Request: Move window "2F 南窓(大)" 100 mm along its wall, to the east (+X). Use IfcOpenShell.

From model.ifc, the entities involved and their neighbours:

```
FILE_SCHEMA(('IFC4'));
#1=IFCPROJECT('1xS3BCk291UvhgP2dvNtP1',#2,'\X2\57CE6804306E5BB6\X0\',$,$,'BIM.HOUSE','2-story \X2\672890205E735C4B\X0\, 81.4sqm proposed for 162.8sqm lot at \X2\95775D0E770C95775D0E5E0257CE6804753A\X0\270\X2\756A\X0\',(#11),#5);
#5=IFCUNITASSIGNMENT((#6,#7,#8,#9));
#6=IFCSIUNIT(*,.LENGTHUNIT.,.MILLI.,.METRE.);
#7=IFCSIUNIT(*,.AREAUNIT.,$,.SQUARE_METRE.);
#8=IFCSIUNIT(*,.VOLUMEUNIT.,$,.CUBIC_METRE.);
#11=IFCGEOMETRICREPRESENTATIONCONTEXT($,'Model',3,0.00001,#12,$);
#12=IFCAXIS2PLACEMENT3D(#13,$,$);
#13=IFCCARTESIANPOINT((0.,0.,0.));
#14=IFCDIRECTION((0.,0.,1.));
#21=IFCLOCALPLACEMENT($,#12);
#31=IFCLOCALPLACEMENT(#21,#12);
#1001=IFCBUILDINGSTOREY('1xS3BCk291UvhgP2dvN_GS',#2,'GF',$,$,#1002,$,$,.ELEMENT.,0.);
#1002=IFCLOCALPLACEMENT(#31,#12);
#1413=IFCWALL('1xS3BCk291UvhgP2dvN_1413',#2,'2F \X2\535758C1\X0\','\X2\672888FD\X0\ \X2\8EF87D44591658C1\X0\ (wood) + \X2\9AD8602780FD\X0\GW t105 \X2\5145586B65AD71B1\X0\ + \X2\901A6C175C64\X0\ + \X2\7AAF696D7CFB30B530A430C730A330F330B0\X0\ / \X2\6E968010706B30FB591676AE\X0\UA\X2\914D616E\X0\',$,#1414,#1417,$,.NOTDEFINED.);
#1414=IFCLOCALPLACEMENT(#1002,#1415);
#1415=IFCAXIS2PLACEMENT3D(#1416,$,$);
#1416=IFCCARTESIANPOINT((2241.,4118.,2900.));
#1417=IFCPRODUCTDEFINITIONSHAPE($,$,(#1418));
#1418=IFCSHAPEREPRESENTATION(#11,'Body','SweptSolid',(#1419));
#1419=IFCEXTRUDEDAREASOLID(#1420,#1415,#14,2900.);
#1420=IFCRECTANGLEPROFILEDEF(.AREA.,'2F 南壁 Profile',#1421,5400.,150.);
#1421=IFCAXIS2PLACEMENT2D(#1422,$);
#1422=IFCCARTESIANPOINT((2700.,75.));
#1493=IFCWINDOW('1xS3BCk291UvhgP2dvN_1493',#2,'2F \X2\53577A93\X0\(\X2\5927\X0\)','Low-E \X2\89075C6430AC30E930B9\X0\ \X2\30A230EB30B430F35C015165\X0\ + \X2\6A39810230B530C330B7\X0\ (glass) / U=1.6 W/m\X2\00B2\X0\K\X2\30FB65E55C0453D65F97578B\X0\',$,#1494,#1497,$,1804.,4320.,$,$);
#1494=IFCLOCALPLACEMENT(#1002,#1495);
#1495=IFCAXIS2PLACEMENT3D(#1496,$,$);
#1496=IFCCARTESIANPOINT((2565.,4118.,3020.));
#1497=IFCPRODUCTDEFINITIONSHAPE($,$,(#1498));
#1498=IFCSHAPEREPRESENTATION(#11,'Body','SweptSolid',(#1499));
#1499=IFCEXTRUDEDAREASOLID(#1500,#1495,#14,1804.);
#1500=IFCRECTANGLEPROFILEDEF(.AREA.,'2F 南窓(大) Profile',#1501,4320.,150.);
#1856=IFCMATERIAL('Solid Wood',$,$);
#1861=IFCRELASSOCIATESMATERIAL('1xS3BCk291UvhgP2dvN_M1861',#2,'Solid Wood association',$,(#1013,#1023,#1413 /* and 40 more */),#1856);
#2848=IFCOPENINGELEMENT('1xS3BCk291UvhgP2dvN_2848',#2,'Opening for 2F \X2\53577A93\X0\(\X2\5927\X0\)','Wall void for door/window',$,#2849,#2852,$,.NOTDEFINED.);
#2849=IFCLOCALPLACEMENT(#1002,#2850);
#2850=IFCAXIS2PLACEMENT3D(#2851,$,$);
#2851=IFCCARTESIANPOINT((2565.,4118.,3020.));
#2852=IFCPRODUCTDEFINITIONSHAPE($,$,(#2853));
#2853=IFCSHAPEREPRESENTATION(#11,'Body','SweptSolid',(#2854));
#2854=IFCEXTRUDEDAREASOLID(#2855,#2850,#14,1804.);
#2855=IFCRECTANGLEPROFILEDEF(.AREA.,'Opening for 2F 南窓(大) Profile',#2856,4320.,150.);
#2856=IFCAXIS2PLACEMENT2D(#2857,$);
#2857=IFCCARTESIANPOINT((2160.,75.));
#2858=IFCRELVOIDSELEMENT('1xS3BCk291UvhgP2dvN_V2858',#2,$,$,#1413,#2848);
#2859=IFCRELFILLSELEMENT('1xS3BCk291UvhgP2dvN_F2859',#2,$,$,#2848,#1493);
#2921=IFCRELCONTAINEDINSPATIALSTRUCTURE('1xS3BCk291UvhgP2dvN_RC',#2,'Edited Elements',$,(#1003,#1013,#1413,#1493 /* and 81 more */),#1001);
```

```python
import ifcopenshell
import ifcopenshell.api.geometry
import ifcopenshell.util.placement
import ifcopenshell.util.unit

model = ifcopenshell.open("model.ifc")
unit_scale = ifcopenshell.util.unit.calculate_unit_scale(model)

window = model.by_guid("1xS3BCk291UvhgP2dvN_1493")
opening = window.FillsVoids[0].RelatingOpeningElement
wall = opening.VoidsElements[0].RelatingBuildingElement

wall_matrix = ifcopenshell.util.placement.get_local_placement(wall.ObjectPlacement)
shift = wall_matrix[:3, 0] * 0.1 / unit_scale
before = ifcopenshell.util.placement.get_local_placement(window.ObjectPlacement)[:3, 3].copy()

# The window is not placed relative to its opening, so move both.
for product in (opening, window):
    matrix = ifcopenshell.util.placement.get_local_placement(product.ObjectPlacement)
    matrix[:3, 3] += shift
    ifcopenshell.api.geometry.edit_object_placement(model, product=product, matrix=matrix, is_si=False)

after = ifcopenshell.util.placement.get_local_placement(window.ObjectPlacement)[:3, 3]
print("window moved by", (after - before).round(3) + 0.0)

model.write("model_updated.ifc")
```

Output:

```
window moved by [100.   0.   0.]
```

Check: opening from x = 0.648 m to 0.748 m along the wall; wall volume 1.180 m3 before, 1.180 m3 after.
